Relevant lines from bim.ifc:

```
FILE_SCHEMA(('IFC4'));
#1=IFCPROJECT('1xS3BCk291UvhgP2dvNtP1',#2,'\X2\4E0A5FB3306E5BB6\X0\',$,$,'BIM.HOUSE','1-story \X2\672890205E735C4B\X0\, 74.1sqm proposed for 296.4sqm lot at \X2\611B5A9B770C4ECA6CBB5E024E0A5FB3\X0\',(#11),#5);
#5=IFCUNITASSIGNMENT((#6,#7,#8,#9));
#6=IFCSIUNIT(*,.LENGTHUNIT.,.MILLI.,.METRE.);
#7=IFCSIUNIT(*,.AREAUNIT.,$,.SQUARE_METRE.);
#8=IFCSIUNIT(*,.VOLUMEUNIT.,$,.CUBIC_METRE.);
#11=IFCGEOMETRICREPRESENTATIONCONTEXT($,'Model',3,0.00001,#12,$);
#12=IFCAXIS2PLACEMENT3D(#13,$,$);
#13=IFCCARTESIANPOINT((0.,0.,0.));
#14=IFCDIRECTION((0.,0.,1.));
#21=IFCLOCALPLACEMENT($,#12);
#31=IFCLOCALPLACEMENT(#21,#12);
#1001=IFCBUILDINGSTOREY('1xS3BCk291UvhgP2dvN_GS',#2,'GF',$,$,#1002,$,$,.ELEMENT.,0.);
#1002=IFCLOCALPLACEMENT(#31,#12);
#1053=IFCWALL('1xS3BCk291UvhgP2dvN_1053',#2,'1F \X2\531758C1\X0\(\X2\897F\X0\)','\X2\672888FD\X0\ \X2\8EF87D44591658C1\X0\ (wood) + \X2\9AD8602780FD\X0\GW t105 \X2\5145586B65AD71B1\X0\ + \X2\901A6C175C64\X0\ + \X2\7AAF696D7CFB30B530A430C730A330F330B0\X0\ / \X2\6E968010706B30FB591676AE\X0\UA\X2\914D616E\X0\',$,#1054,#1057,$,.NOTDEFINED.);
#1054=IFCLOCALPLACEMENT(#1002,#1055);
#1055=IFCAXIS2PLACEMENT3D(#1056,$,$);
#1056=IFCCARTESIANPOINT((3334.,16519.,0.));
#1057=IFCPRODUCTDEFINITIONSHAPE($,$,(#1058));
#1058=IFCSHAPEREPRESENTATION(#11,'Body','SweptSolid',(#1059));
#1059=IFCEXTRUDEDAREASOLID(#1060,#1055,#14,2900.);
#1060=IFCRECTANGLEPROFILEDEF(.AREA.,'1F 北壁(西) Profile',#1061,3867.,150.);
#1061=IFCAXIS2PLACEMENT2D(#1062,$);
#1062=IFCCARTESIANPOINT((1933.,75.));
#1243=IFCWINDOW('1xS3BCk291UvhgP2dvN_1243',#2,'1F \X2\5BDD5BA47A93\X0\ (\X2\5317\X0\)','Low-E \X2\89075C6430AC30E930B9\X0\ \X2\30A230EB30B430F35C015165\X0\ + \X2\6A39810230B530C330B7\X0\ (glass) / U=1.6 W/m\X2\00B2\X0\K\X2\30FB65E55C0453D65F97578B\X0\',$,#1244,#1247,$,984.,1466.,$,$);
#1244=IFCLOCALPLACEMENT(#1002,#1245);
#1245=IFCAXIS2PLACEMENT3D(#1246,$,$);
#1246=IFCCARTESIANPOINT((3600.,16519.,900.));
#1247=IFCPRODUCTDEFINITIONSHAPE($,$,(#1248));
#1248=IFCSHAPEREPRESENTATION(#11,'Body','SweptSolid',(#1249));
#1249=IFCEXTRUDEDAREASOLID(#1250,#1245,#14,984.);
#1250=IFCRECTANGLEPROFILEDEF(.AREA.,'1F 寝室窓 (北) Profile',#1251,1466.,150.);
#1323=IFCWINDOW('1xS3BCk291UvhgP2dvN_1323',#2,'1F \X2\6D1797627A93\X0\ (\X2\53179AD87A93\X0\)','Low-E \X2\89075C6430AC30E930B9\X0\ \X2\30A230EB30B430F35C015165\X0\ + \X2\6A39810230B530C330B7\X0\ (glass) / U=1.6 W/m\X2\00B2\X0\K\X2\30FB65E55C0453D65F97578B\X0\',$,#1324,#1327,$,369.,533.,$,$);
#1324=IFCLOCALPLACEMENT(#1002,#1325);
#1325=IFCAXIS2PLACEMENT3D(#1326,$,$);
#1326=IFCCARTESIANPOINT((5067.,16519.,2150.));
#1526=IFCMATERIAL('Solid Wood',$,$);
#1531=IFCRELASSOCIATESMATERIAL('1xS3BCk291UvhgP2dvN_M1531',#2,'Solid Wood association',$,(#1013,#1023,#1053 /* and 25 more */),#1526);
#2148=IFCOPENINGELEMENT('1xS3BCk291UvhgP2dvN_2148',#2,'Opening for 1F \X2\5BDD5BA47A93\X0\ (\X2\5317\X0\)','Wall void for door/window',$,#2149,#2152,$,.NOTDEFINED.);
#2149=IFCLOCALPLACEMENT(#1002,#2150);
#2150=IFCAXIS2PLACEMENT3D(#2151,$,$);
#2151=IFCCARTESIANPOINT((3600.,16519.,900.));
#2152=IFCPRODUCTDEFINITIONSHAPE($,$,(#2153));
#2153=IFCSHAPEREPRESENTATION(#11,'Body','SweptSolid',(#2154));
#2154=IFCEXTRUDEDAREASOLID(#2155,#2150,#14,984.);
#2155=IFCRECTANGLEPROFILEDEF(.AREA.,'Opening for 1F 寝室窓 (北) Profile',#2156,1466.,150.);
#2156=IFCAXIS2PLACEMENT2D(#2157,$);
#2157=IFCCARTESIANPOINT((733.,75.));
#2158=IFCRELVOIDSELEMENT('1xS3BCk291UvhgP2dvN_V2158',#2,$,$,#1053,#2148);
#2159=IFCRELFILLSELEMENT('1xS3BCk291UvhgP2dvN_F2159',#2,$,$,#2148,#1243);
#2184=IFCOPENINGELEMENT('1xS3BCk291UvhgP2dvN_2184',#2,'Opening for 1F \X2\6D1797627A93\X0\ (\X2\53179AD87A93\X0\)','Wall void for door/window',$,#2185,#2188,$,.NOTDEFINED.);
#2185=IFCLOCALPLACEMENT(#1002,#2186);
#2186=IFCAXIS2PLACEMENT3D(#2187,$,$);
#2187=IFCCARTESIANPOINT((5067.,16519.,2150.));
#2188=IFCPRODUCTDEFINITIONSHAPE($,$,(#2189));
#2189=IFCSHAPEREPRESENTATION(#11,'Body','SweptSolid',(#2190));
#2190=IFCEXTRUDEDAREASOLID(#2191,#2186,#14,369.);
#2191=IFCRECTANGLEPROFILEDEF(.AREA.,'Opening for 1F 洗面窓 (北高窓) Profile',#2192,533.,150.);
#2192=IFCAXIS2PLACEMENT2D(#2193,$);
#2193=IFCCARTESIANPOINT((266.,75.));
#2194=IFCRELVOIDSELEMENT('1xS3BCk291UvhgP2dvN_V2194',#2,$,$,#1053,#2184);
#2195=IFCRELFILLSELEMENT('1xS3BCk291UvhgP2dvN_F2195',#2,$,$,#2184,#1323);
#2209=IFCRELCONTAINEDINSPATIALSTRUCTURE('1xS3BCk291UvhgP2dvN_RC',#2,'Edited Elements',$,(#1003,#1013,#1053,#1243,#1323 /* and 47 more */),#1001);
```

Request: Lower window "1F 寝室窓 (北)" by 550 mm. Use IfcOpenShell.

```python
import numpy as np
import ifcopenshell
import ifcopenshell.api.geometry
import ifcopenshell.util.placement
import ifcopenshell.util.unit

model = ifcopenshell.open("bim.ifc")
unit_scale = ifcopenshell.util.unit.calculate_unit_scale(model)

window = model.by_id(1243)
opening = window.FillsVoids[0].RelatingOpeningElement
dz = -0.55 / unit_scale

shift = np.array([0.0, 0.0, dz])
# The window is not placed relative to its opening, so move both.
for product in (opening, window):
    matrix = ifcopenshell.util.placement.get_local_placement(product.ObjectPlacement)
    matrix[:3, 3] += shift
    ifcopenshell.api.geometry.edit_object_placement(model, product=product, matrix=matrix, is_si=False)

print(f"moved by {dz * unit_scale:+.3f} m")

model.write("bim_rev.ifc")
```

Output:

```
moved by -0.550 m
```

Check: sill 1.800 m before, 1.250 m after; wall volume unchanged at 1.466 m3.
